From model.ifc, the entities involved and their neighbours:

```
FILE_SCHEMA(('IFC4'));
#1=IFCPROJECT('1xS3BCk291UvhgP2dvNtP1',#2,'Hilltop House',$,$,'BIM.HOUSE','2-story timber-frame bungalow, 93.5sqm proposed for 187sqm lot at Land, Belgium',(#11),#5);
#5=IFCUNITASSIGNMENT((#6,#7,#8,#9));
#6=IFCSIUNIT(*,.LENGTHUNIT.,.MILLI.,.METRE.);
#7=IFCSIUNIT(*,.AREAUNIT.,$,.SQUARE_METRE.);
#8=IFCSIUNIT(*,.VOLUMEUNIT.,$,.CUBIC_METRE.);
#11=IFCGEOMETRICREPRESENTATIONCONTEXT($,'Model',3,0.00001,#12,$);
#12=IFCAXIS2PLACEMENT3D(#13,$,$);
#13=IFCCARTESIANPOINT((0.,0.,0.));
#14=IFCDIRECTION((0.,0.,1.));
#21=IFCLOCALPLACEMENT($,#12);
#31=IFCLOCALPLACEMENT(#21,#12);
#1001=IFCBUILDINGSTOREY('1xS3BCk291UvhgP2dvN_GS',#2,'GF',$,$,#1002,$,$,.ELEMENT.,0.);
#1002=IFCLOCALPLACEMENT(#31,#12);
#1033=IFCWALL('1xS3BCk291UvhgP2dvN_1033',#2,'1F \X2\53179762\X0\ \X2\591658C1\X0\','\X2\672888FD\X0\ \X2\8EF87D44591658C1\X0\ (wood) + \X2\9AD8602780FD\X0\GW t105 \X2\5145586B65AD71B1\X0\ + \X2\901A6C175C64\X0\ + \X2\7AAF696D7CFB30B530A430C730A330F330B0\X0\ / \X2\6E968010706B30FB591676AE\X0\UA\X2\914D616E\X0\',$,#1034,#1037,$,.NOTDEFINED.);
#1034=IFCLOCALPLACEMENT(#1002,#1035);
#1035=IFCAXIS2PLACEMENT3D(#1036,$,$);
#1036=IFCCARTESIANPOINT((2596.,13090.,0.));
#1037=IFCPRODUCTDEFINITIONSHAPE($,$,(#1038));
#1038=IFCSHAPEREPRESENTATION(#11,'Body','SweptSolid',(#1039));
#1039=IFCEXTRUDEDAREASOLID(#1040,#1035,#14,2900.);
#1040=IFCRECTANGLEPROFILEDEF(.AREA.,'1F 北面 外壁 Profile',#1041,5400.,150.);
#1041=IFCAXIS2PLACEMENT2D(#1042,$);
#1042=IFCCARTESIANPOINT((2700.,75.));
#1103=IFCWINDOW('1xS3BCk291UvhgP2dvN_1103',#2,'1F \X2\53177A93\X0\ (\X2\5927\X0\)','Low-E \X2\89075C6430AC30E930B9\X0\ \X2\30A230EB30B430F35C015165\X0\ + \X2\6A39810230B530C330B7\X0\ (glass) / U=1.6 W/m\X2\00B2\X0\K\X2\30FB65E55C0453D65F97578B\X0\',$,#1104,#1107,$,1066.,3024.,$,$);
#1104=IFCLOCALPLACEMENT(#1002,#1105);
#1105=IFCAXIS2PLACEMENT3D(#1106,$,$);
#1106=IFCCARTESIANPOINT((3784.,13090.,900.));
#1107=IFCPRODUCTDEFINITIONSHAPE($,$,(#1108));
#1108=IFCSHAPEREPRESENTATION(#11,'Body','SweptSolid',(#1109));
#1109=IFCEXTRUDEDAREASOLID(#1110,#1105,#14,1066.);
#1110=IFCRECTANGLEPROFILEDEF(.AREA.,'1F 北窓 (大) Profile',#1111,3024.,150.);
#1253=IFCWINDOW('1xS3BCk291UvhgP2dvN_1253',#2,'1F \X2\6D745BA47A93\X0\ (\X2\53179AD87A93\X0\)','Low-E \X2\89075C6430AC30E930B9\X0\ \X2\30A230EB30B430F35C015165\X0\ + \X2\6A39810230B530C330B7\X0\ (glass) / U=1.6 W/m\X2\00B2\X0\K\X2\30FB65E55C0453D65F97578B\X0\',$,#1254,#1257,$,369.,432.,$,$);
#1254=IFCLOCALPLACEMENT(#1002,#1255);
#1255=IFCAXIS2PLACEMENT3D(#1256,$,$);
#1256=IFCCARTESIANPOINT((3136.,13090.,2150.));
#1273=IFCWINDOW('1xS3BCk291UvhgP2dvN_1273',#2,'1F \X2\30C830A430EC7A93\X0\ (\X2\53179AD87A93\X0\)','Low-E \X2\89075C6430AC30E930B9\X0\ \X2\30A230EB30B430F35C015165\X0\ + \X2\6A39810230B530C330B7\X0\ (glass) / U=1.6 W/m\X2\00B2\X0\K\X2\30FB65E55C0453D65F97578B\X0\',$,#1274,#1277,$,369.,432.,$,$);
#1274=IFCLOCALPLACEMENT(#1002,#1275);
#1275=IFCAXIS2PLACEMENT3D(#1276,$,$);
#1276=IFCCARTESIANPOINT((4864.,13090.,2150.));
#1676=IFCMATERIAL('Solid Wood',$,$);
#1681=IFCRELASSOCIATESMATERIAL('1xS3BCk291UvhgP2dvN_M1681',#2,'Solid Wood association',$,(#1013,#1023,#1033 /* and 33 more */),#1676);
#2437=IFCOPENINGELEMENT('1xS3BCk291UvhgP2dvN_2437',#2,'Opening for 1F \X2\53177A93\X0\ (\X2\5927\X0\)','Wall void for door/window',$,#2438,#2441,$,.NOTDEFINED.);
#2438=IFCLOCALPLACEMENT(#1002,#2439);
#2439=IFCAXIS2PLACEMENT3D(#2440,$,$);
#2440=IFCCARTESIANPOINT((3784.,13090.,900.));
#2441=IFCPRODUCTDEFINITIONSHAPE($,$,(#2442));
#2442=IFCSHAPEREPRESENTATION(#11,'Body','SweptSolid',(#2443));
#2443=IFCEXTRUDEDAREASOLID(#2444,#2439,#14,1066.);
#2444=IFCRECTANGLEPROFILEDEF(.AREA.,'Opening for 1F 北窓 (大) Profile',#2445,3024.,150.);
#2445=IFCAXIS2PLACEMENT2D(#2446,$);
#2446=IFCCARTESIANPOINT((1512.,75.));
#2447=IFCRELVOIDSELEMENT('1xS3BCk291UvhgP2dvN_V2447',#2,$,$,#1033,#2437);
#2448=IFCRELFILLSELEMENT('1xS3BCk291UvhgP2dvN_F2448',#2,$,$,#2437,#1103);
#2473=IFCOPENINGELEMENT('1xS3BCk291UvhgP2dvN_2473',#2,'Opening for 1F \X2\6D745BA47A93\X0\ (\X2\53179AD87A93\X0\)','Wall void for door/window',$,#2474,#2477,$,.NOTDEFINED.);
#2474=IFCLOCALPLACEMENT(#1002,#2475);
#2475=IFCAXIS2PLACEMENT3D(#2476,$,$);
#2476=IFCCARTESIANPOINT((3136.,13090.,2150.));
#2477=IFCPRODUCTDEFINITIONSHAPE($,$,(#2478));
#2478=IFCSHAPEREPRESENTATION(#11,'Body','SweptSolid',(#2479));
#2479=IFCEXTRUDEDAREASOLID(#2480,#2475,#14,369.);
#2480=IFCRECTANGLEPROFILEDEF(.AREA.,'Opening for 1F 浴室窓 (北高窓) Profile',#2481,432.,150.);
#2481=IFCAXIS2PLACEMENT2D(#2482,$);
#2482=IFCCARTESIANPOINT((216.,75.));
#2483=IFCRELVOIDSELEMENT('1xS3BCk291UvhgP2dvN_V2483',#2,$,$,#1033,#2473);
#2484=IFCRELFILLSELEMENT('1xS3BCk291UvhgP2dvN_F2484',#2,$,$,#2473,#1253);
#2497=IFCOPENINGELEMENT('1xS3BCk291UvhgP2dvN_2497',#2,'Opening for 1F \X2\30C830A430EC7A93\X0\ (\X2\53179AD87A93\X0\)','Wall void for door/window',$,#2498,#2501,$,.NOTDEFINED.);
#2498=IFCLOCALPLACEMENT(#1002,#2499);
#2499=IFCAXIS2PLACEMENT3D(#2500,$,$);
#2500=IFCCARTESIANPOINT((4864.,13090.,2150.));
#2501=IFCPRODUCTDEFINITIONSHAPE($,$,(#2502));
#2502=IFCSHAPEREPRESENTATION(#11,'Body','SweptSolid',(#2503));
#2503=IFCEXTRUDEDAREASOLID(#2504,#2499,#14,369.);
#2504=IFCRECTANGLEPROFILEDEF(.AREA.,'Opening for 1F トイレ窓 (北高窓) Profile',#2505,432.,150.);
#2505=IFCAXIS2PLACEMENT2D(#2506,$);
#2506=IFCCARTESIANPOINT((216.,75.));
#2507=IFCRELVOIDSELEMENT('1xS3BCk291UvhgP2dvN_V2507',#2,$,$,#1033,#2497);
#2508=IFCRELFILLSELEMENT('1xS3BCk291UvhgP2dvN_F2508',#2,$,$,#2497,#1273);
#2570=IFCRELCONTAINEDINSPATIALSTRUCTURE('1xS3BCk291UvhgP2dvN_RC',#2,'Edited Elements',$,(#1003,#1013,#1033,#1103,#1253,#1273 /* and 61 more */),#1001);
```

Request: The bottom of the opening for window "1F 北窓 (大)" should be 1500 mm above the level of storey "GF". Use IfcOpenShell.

```python
import numpy as np
import ifcopenshell
import ifcopenshell.api.geometry
import ifcopenshell.geom
import ifcopenshell.util.element
import ifcopenshell.util.placement
import ifcopenshell.util.shape
import ifcopenshell.util.unit

model = ifcopenshell.open("model.ifc")
unit_scale = ifcopenshell.util.unit.calculate_unit_scale(model)

window = model.by_guid("1xS3BCk291UvhgP2dvN_1103")
opening = window.FillsVoids[0].RelatingOpeningElement
storey = ifcopenshell.util.element.get_container(window, ifc_class="IfcBuildingStorey")
level = ifcopenshell.util.placement.get_local_placement(storey.ObjectPlacement)[2, 3]

# The opening's origin need not be at the sill, so measure its lowest point.
shape = ifcopenshell.geom.create_shape(ifcopenshell.geom.settings(), opening)
bottom = ifcopenshell.util.shape.get_shape_bottom_elevation(shape, shape.geometry) / unit_scale
dz = level + 1500.0 - bottom

shift = np.array([0.0, 0.0, dz])
# The window is not placed relative to its opening, so move both.
for product in (opening, window):
    matrix = ifcopenshell.util.placement.get_local_placement(product.ObjectPlacement)
    matrix[:3, 3] += shift
    ifcopenshell.api.geometry.edit_object_placement(model, product=product, matrix=matrix, is_si=False)

print(f"moved by {dz * unit_scale:+.3f} m")

model.write("model_updated.ifc")
```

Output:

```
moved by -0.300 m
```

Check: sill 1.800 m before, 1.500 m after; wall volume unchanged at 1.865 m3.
